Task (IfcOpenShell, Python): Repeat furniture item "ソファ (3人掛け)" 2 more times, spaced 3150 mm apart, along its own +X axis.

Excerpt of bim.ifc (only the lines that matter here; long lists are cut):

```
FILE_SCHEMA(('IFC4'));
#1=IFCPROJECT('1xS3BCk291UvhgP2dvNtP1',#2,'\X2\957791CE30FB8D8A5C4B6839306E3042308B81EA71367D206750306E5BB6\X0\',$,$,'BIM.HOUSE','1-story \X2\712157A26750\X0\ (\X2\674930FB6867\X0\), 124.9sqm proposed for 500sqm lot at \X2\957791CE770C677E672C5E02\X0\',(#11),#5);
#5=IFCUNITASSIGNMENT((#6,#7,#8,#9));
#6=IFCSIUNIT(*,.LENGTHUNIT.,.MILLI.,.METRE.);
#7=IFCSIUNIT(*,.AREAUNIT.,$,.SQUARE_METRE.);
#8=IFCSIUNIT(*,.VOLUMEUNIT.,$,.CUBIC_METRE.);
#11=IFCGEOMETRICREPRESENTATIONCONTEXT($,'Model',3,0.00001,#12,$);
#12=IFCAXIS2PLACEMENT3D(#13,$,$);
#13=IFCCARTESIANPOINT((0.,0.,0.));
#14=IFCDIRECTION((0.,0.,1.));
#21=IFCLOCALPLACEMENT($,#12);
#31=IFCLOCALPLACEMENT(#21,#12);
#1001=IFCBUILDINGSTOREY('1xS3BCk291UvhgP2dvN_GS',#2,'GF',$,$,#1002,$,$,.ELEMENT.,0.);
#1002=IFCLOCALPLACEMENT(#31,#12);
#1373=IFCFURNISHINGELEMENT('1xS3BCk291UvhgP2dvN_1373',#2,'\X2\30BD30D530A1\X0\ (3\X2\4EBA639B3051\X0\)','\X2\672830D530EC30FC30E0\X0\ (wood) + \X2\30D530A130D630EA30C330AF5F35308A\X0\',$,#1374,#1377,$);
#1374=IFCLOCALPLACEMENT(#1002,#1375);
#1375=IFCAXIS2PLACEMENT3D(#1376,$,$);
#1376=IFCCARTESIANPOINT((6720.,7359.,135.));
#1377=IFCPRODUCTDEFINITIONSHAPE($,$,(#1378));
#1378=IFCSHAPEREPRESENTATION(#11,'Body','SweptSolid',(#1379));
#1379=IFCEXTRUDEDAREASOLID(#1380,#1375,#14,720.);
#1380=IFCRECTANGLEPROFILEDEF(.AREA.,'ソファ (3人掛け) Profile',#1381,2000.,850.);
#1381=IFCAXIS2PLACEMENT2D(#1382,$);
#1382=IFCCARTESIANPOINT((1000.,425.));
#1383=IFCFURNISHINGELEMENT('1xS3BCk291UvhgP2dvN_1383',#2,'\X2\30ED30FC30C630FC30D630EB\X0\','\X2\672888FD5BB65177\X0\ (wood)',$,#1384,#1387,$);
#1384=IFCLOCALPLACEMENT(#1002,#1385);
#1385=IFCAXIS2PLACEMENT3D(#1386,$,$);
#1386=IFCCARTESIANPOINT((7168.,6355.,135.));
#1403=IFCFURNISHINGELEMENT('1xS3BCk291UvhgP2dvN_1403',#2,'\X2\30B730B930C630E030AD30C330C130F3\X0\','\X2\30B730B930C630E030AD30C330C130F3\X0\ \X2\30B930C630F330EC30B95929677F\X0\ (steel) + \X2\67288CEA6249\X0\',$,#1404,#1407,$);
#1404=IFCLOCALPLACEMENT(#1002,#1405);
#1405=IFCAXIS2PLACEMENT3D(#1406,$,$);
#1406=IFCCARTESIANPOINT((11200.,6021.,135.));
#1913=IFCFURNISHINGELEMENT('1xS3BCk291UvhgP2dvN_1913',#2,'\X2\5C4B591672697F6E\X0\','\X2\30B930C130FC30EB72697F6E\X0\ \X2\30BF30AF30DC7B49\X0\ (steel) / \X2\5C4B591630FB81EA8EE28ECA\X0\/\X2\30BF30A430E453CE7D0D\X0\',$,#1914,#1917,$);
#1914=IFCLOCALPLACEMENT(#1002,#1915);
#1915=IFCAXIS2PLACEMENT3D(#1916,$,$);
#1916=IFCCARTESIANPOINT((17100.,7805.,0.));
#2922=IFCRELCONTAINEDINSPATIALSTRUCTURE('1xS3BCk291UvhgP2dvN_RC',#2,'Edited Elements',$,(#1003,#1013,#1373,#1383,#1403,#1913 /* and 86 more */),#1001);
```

```python
import ifcopenshell
import ifcopenshell.api.geometry
import ifcopenshell.api.root
import ifcopenshell.util.element
import ifcopenshell.util.placement
import ifcopenshell.util.unit

model = ifcopenshell.open("bim.ifc")
unit_scale = ifcopenshell.util.unit.calculate_unit_scale(model)


def reuse_history(source, copy):
    """copy_class also copies each property set's owner history, people and application; keep the originals."""
    for rel in copy.IsDefinedBy:
        if rel.is_a("IfcRelDefinesByProperties") and (history := rel.RelatingPropertyDefinition.OwnerHistory):
            rel.RelatingPropertyDefinition.OwnerHistory = source.OwnerHistory
            ifcopenshell.util.element.remove_deep2(model, history)


source = model.by_guid("1xS3BCk291UvhgP2dvN_1373")
base = ifcopenshell.util.placement.get_local_placement(source.ObjectPlacement)
step = base[:3, 0] * 3.15 / unit_scale

for i in range(1, 3):
    copy = ifcopenshell.api.root.copy_class(model, product=source)
    copy.Representation = ifcopenshell.util.element.copy_deep(
        model, source.Representation, exclude=["IfcGeometricRepresentationContext", "IfcRepresentationMap"]
    )
    reuse_history(source, copy)
    matrix = base.copy()
    matrix[:3, 3] += i * step
    print("added at", matrix[:3, 3].round(3) + 0.0)
    ifcopenshell.api.geometry.edit_object_placement(model, product=copy, matrix=matrix, is_si=False)

model.write("bim_updated.ifc")
```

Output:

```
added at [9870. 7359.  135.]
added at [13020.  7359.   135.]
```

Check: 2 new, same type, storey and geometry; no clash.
